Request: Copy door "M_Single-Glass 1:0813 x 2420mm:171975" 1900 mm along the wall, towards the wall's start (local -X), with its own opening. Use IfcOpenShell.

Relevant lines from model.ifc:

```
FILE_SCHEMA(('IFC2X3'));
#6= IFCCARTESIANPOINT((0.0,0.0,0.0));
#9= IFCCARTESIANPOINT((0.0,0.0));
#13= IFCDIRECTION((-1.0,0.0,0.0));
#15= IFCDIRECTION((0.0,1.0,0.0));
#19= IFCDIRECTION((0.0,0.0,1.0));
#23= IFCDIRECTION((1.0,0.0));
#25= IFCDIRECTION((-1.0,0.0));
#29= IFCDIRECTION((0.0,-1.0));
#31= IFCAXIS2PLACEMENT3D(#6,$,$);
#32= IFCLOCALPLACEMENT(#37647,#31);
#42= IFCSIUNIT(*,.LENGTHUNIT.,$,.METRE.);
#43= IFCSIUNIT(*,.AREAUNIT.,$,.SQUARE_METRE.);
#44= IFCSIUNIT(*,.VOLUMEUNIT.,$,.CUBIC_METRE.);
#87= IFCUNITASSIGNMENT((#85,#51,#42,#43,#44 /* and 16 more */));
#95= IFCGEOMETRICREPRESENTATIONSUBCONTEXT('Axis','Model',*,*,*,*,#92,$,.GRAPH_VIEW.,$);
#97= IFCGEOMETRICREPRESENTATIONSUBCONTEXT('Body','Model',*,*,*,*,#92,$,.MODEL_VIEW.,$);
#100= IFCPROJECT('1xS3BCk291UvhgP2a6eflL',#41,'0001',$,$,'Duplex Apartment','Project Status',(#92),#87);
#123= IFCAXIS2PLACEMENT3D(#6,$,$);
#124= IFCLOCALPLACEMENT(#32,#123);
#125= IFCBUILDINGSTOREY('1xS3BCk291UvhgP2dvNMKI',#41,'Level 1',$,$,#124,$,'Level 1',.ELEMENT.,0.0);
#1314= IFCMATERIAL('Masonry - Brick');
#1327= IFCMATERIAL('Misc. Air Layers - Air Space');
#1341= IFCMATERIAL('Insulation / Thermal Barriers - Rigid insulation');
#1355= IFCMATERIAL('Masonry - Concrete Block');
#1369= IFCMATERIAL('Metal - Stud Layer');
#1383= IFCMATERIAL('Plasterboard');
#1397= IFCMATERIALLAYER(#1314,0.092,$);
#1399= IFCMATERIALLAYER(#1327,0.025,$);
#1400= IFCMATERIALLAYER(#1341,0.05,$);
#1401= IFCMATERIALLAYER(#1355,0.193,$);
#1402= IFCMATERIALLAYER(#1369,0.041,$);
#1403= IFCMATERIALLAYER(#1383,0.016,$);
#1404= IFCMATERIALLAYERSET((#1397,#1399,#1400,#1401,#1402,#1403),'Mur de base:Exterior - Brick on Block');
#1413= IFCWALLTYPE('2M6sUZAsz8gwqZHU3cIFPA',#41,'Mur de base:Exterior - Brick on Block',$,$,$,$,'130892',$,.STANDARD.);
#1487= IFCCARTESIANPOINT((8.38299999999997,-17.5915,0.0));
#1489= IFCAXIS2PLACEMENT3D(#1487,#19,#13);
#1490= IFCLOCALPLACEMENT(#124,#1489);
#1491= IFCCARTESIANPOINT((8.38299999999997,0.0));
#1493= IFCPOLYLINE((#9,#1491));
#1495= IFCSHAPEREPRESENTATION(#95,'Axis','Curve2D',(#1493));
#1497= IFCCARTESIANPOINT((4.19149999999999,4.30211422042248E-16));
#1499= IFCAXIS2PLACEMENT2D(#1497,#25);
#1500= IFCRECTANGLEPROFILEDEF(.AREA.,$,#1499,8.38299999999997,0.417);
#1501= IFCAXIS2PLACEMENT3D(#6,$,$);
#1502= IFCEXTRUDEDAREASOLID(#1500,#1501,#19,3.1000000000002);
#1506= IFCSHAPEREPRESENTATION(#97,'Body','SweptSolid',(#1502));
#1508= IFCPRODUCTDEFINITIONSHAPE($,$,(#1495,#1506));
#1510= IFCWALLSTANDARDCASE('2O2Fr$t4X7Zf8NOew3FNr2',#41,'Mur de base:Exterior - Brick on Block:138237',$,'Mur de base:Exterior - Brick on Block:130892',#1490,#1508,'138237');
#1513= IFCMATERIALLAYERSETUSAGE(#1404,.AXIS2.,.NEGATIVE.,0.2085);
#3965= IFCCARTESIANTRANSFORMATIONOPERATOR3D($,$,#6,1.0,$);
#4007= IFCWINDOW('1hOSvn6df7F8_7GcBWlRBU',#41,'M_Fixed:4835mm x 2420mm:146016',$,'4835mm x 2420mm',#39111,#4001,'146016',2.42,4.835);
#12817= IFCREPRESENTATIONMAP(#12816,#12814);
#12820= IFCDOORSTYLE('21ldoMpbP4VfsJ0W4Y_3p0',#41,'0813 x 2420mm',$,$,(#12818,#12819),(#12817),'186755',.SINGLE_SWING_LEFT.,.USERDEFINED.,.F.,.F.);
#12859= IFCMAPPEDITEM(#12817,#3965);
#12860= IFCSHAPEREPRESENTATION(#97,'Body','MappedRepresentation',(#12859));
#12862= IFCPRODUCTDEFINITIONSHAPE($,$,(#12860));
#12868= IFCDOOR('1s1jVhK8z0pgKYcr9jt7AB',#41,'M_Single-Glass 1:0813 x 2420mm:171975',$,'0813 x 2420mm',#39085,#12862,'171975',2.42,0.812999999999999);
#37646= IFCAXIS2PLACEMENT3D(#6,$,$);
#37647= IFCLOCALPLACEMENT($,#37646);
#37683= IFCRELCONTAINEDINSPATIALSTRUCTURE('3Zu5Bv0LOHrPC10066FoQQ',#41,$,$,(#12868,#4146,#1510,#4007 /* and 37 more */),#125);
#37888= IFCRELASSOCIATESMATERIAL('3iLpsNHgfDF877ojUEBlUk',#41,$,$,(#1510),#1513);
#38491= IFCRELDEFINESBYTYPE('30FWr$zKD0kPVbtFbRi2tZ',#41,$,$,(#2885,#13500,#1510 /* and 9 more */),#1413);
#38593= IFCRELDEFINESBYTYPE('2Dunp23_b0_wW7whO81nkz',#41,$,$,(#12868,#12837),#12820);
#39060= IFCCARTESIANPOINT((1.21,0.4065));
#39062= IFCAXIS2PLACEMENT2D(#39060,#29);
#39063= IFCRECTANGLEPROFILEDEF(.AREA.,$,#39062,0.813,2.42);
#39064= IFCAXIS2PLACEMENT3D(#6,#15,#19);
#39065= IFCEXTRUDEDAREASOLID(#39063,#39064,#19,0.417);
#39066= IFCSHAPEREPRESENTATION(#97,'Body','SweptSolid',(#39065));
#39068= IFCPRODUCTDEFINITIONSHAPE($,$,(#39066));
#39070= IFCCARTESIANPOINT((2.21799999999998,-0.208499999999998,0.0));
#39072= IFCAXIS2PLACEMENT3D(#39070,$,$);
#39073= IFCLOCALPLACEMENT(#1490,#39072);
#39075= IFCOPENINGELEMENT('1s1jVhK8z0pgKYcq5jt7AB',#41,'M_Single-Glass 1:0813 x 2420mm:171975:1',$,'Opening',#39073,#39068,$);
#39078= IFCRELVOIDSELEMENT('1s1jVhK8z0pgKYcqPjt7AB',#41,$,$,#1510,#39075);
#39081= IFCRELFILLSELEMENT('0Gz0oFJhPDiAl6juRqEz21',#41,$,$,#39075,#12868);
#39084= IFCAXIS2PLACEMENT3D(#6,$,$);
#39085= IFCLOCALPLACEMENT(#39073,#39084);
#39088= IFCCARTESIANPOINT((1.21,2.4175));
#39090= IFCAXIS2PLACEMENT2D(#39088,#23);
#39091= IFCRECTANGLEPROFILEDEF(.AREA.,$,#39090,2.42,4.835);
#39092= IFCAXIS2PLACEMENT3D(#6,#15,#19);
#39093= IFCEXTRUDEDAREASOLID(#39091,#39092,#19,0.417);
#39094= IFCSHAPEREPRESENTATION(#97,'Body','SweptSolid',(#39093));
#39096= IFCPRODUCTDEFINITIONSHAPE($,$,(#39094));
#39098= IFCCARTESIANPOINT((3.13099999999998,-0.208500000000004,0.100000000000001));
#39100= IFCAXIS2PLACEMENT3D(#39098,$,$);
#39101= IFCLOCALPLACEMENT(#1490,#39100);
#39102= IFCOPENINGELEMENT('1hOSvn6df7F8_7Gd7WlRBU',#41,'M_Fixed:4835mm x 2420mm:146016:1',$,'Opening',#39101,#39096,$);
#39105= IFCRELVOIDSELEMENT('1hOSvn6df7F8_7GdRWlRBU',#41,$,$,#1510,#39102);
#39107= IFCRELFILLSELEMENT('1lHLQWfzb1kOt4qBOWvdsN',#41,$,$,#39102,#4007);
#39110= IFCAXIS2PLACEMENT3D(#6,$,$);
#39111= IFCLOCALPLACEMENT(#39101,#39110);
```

```python
import ifcopenshell
import ifcopenshell.api.feature
import ifcopenshell.api.geometry
import ifcopenshell.api.root
import ifcopenshell.geom
import ifcopenshell.util.element
import ifcopenshell.util.placement
import ifcopenshell.util.shape
import ifcopenshell.util.unit

model = ifcopenshell.open("model.ifc")
unit_scale = ifcopenshell.util.unit.calculate_unit_scale(model)
settings = ifcopenshell.geom.settings()


def volume(element):
    """Net volume in cubic metres, openings subtracted."""
    shape = ifcopenshell.geom.create_shape(settings, element)
    return ifcopenshell.util.shape.get_volume(shape.geometry)


def reuse_history(source, copy):
    """copy_class also copies each property set's owner history, people and application; keep the originals."""
    for rel in copy.IsDefinedBy:
        if rel.is_a("IfcRelDefinesByProperties") and (history := rel.RelatingPropertyDefinition.OwnerHistory):
            rel.RelatingPropertyDefinition.OwnerHistory = source.OwnerHistory
            ifcopenshell.util.element.remove_deep2(model, history)


door = model.by_id(12868)
opening = door.FillsVoids[0].RelatingOpeningElement
wall = opening.VoidsElements[0].RelatingBuildingElement
before = volume(wall)
shift = ifcopenshell.util.placement.get_local_placement(wall.ObjectPlacement)[:3, 0] * -1.9 / unit_scale

# copy_class copies the void relationship, type, container and properties, but no geometry.
new_opening = ifcopenshell.api.root.copy_class(model, product=opening)
new_opening.Representation = ifcopenshell.util.element.copy_deep(
    model, opening.Representation, exclude=["IfcGeometricRepresentationContext", "IfcRepresentationMap"]
)
new_opening.Name = "M_Single-Glass 1:0813 x 2420mm"
new_door = ifcopenshell.api.root.copy_class(model, product=door)
new_door.Representation = ifcopenshell.util.element.copy_deep(
    model, door.Representation, exclude=["IfcGeometricRepresentationContext", "IfcRepresentationMap"]
)
new_door.Name = "M_Single-Glass 1:0813 x 2420mm"
new_door.Tag = None
reuse_history(door, new_door)
fills = ifcopenshell.api.feature.add_filling(model, opening=new_opening, element=new_door)
fills.OwnerHistory = new_door.OwnerHistory  # required in IFC2X3

for old, new in ((opening, new_opening), (door, new_door)):
    matrix = ifcopenshell.util.placement.get_local_placement(old.ObjectPlacement)
    matrix[:3, 3] += shift
    ifcopenshell.api.geometry.edit_object_placement(model, product=new, matrix=matrix, is_si=False)

after = volume(wall)

print(f"wall volume {before:.3f} -> {after:.3f} m3")

model.write("model_rev.ifc")
```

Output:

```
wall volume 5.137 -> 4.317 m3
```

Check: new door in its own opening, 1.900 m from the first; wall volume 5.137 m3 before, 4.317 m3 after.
